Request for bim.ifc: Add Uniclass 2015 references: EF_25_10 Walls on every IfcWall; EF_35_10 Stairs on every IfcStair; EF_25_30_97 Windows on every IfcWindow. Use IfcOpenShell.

First a look at what the model holds.

```python
import ifcopenshell

model = ifcopenshell.open("bim.ifc")
print(model.schema)
print("classifications:", [c.Name for c in model.by_type("IfcClassification")])
for ifc_class in ("IfcDoor", "IfcRoof", "IfcStair", "IfcWall", "IfcWindow"):
    print(ifc_class, len(model.by_type(ifc_class)))
```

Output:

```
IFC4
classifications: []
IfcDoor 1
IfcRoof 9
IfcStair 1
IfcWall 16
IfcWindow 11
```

```python
import ifcopenshell
import ifcopenshell.api.classification

model = ifcopenshell.open("bim.ifc")

system = ifcopenshell.api.classification.add_classification(model, classification="Uniclass 2015")

codes = {
    "IfcWall": ("EF_25_10", "Walls"),
    "IfcStair": ("EF_35_10", "Stairs"),
    "IfcWindow": ("EF_25_30_97", "Windows"),
}
for ifc_class, (code, name) in codes.items():
    products = model.by_type(ifc_class)
    ifcopenshell.api.classification.add_reference(
        model, products=products, classification=system, identification=code, name=name
    )
    print(code, len(products))

model.write("bim_rev.ifc")
```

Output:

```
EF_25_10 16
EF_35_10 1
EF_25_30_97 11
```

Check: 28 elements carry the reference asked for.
